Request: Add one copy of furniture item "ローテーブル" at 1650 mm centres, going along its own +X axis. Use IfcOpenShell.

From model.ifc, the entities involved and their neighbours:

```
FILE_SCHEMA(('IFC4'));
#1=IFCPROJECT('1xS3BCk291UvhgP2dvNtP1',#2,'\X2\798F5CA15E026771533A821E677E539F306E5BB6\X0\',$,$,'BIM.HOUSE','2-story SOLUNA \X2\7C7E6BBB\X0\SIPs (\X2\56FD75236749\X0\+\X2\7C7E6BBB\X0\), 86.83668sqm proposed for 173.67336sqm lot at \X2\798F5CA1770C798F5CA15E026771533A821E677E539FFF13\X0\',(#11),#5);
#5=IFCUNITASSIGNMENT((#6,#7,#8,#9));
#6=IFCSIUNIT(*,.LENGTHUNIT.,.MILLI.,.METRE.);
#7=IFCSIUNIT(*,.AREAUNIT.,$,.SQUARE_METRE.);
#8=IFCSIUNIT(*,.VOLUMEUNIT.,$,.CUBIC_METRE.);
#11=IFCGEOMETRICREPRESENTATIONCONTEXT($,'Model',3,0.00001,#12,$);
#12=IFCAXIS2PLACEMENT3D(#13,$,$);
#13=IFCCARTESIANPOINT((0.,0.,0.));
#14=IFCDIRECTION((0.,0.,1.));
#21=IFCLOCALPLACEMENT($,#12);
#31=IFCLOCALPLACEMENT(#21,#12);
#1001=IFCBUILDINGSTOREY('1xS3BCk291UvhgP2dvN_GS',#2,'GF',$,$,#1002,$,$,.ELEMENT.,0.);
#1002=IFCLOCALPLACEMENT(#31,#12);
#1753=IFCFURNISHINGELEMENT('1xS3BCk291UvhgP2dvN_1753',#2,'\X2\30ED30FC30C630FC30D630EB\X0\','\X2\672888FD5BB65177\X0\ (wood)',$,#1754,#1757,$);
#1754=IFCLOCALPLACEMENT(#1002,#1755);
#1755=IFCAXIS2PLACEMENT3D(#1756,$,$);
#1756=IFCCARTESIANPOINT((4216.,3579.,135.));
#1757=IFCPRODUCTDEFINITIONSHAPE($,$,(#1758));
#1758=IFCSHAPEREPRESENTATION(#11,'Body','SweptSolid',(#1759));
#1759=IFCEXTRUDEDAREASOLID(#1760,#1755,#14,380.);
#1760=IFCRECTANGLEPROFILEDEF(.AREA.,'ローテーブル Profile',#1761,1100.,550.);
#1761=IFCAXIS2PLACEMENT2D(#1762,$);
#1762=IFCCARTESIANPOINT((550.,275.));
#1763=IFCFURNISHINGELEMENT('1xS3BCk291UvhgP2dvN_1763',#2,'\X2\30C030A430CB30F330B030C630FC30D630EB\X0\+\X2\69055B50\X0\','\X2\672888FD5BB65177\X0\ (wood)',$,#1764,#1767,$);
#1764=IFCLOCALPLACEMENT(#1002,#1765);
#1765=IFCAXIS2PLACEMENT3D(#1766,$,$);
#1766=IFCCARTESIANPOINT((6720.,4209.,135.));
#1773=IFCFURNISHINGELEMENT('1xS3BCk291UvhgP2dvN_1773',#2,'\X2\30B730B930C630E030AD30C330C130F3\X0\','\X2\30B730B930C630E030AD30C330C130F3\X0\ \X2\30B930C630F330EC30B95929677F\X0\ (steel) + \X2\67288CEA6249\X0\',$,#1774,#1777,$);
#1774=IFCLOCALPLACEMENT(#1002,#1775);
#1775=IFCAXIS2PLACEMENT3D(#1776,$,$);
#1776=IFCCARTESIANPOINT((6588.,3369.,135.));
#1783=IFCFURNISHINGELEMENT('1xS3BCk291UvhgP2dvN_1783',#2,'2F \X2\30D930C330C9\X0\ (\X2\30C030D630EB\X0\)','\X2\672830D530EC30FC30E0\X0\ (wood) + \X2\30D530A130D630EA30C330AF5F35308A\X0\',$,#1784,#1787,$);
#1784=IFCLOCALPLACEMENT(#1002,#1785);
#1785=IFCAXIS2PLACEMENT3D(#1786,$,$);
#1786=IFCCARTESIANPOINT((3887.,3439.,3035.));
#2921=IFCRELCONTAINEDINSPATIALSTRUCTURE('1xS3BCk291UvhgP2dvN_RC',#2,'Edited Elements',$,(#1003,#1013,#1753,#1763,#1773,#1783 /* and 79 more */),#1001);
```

```python
import ifcopenshell
import ifcopenshell.api.geometry
import ifcopenshell.api.root
import ifcopenshell.util.element
import ifcopenshell.util.placement

model = ifcopenshell.open("model.ifc")


def reuse_history(source, copy):
    """copy_class also copies each property set's owner history, people and application; keep the originals."""
    for rel in copy.IsDefinedBy:
        if rel.is_a("IfcRelDefinesByProperties") and (history := rel.RelatingPropertyDefinition.OwnerHistory):
            rel.RelatingPropertyDefinition.OwnerHistory = source.OwnerHistory
            ifcopenshell.util.element.remove_deep2(model, history)


source = model.by_guid("1xS3BCk291UvhgP2dvN_1753")
base = ifcopenshell.util.placement.get_local_placement(source.ObjectPlacement)
step = base[:3, 0] * 1650.0

for i in range(1, 2):
    copy = ifcopenshell.api.root.copy_class(model, product=source)
    copy.Representation = ifcopenshell.util.element.copy_deep(
        model, source.Representation, exclude=["IfcGeometricRepresentationContext", "IfcRepresentationMap"]
    )
    reuse_history(source, copy)
    matrix = base.copy()
    matrix[:3, 3] += i * step
    print("added at", matrix[:3, 3].round(3) + 0.0)
    ifcopenshell.api.geometry.edit_object_placement(model, product=copy, matrix=matrix, is_si=False)

model.write("model_v2.ifc")
```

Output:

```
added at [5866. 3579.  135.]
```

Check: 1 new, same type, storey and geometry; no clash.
